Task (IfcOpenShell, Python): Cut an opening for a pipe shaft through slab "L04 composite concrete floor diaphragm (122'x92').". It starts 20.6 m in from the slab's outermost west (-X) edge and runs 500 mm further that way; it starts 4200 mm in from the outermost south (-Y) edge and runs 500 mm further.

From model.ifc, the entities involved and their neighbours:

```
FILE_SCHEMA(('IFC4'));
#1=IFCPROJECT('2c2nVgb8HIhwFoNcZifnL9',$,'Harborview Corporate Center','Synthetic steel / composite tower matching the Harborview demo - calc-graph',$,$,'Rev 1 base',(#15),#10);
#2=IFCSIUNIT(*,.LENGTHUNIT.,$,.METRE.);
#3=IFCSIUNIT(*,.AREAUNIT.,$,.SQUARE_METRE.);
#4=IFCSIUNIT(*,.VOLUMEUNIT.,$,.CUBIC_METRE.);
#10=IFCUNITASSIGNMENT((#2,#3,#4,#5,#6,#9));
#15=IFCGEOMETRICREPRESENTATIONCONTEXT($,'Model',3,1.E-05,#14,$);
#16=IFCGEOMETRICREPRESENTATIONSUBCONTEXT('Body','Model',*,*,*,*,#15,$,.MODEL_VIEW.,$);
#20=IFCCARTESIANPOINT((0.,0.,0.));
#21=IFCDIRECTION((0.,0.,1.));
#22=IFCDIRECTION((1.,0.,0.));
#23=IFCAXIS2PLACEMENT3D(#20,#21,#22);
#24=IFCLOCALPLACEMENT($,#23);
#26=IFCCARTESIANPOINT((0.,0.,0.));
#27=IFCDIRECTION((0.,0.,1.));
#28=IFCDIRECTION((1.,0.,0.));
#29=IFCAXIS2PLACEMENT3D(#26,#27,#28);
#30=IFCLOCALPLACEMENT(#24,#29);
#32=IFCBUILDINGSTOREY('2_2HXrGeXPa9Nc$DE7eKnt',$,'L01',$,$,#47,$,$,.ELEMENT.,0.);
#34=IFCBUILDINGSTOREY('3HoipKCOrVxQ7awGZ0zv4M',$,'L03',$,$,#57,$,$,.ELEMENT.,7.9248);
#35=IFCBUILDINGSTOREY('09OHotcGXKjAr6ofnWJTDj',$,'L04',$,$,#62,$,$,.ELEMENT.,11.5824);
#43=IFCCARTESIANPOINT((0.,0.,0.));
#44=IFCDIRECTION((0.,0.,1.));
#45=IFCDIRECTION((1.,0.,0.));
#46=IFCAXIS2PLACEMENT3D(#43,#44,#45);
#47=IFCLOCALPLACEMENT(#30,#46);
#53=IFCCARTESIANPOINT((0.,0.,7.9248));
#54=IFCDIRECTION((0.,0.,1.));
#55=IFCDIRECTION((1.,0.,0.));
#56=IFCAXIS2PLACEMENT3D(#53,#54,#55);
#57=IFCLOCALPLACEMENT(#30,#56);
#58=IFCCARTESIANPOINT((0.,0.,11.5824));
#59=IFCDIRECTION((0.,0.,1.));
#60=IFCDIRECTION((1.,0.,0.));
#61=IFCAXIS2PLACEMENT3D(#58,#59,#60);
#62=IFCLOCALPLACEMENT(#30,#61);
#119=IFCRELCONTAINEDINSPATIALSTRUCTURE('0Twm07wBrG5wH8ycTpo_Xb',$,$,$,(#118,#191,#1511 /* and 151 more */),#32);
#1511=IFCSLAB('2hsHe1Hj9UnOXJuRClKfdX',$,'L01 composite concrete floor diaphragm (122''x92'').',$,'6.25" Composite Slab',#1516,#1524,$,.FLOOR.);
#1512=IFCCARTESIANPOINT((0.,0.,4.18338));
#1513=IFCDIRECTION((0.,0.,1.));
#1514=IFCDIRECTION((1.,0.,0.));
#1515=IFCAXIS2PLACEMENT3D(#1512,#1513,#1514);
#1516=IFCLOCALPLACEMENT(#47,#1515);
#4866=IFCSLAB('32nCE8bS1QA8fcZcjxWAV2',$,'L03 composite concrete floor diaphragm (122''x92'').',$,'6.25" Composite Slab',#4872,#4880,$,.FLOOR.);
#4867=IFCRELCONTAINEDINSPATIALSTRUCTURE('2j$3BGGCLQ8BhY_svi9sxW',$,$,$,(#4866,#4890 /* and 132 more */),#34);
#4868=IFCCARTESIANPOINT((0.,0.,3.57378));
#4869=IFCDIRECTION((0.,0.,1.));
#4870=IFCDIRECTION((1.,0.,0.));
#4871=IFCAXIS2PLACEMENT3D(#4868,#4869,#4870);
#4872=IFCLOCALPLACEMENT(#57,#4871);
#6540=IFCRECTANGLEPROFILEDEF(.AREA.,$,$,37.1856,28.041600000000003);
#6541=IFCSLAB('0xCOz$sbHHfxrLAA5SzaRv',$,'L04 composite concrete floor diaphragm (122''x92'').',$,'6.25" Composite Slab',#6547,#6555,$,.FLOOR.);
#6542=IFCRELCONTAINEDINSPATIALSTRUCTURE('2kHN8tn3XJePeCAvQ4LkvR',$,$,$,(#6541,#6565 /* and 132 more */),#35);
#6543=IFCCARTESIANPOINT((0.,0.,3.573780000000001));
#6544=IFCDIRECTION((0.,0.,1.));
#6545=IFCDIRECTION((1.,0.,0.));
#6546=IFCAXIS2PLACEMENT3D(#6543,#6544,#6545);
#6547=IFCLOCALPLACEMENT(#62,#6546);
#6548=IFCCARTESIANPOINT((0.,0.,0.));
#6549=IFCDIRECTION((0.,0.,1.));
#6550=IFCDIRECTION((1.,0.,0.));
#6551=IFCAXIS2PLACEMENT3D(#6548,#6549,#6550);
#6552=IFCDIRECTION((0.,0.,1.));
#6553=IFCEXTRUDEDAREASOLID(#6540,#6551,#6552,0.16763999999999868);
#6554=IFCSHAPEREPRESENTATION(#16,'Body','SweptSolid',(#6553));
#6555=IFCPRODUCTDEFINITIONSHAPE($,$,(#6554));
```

```python
import numpy as np
import ifcopenshell
import ifcopenshell.api.feature
import ifcopenshell.api.geometry
import ifcopenshell.api.root
import ifcopenshell.geom
import ifcopenshell.util.placement
import ifcopenshell.util.representation
import ifcopenshell.util.shape
import ifcopenshell.util.unit

model = ifcopenshell.open("model.ifc")
unit_scale = ifcopenshell.util.unit.calculate_unit_scale(model)
settings = ifcopenshell.geom.settings()


def volume(element):
    """Net volume in cubic metres, openings subtracted."""
    shape = ifcopenshell.geom.create_shape(settings, element)
    return ifcopenshell.util.shape.get_volume(shape.geometry)


slab = model.by_guid("0xCOz$sbHHfxrLAA5SzaRv")
before = volume(slab)

# Extent in the slab's own axes, in metres. The edges named are its -X and -Y sides.
slab_shape = ifcopenshell.geom.create_shape(settings, slab)
vertices = ifcopenshell.util.shape.get_vertices(slab_shape.geometry)
x_min, y_min, bottom = vertices.min(axis=0)
top = vertices[:, 2].max()

opening = ifcopenshell.api.root.create_entity(model, ifc_class="IfcOpeningElement", name="Pipe shaft opening", predefined_type="OPENING")
context = ifcopenshell.util.representation.get_context(model, "Model", "Body", "MODEL_VIEW")
width, depth = 0.5, 0.5
outline = [(0.0, 0.0), (width, 0.0), (width, depth), (0.0, depth), (0.0, 0.0)]
# Overshoot both faces by 50 mm so the cut is clean.
shape = ifcopenshell.api.geometry.add_slab_representation(
    model, context=context, depth=top - bottom + 0.1, polyline=outline
)
ifcopenshell.api.geometry.assign_representation(model, product=opening, representation=shape)

matrix = ifcopenshell.util.placement.get_local_placement(slab.ObjectPlacement)
matrix[:, 3] = matrix @ np.append(np.array([x_min + 20.6, y_min + 4.2, bottom - 0.05]) / unit_scale, 1.0)
ifcopenshell.api.geometry.edit_object_placement(model, product=opening, matrix=matrix, is_si=False)
ifcopenshell.api.feature.add_feature(model, feature=opening, element=slab)

after = volume(slab)

print(f"slab volume {before:.3f} -> {after:.3f} m3")

model.write("model_updated.ifc")
```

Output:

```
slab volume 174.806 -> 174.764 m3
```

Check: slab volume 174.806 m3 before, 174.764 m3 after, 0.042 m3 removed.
